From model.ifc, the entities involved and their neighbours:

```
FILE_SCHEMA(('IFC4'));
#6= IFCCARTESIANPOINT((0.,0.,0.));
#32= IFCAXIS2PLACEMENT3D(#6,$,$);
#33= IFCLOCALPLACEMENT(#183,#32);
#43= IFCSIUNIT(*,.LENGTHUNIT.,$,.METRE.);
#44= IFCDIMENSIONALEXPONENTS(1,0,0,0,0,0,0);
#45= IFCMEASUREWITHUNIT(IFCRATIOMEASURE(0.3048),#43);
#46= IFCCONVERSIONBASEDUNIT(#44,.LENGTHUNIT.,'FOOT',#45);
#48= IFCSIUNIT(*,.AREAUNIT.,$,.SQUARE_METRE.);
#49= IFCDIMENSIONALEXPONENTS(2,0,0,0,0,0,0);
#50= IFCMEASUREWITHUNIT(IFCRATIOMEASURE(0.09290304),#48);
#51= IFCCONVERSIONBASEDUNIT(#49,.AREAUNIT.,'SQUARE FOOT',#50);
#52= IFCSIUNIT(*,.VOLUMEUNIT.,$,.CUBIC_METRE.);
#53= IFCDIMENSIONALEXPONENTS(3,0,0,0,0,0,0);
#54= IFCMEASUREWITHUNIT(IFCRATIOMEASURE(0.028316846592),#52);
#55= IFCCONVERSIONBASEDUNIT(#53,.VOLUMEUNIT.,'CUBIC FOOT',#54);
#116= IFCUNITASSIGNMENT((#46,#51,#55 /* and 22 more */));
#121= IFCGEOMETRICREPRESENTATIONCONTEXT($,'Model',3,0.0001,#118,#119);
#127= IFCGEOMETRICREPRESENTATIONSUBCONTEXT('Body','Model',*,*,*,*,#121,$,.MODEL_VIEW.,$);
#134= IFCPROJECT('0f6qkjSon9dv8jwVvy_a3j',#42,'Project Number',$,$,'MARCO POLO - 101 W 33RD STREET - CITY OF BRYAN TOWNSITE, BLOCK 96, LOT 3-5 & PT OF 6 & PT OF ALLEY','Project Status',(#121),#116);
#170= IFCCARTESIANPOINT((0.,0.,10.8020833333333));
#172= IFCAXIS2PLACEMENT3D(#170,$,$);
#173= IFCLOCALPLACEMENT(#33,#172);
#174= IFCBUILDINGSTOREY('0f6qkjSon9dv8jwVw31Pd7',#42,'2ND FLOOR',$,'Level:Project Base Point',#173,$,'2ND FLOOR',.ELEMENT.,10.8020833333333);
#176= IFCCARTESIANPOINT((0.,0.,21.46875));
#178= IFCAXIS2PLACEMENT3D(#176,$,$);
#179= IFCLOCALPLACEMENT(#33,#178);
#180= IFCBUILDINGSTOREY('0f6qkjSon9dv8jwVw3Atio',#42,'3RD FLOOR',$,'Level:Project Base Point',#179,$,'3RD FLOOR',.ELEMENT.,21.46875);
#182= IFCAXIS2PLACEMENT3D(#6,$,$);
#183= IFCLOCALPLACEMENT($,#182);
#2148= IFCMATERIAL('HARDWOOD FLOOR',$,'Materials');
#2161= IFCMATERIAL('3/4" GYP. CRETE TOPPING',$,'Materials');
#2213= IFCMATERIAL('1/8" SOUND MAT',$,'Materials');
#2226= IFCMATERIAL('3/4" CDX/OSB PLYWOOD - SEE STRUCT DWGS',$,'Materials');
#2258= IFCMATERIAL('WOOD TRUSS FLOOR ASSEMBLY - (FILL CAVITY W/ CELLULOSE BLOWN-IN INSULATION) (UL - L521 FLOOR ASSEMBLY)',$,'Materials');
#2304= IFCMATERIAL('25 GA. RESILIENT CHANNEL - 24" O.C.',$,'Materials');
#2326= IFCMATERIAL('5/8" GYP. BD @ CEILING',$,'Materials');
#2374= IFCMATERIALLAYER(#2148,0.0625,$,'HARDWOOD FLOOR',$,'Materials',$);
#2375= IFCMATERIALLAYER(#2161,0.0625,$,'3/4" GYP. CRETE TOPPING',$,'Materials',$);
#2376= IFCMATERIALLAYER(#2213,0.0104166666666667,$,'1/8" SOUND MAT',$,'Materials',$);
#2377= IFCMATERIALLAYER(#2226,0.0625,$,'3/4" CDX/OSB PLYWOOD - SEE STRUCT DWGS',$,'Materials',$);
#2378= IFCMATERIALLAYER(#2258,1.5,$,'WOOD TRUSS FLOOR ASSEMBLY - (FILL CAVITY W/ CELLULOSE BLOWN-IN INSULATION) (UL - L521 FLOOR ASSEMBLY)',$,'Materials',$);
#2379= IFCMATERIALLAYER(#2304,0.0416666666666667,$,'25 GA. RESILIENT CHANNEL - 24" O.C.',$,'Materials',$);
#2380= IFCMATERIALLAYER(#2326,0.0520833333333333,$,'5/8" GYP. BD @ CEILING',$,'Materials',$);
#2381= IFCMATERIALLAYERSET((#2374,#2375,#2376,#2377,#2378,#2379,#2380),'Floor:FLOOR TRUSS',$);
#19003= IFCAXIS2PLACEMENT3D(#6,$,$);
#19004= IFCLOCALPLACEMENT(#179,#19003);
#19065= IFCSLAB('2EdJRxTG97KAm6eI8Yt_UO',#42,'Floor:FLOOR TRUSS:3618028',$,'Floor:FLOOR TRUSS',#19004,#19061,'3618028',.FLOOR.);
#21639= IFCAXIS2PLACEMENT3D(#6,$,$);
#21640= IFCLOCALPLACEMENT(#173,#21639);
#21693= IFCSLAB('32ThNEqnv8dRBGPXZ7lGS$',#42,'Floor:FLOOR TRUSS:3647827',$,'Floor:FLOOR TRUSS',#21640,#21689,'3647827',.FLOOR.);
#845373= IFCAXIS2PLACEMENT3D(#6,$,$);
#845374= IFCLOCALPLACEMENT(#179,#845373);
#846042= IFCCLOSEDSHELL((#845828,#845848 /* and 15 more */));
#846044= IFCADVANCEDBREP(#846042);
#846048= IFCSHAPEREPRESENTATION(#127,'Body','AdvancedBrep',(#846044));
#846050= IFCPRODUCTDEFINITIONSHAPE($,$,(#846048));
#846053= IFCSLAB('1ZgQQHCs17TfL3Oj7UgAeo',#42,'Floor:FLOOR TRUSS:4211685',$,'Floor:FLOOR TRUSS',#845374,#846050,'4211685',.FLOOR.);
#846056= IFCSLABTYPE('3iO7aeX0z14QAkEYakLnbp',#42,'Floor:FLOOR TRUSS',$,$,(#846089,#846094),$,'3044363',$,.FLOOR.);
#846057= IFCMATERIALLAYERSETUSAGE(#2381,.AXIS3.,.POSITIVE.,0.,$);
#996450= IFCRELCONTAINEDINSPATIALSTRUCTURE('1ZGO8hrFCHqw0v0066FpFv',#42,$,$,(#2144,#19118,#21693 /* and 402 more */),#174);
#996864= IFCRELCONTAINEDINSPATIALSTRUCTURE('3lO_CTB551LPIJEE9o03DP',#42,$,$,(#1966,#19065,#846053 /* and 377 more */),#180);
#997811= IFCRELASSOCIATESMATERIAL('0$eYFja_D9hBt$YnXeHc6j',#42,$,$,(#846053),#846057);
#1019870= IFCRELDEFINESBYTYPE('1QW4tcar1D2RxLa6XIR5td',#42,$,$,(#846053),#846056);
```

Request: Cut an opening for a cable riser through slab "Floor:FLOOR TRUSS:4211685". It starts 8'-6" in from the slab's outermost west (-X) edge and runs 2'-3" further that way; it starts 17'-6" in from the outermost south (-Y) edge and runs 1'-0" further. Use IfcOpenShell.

```python
import numpy as np
import ifcopenshell
import ifcopenshell.api.feature
import ifcopenshell.api.geometry
import ifcopenshell.api.root
import ifcopenshell.geom
import ifcopenshell.util.placement
import ifcopenshell.util.representation
import ifcopenshell.util.shape
import ifcopenshell.util.unit

model = ifcopenshell.open("model.ifc")
unit_scale = ifcopenshell.util.unit.calculate_unit_scale(model)
settings = ifcopenshell.geom.settings()


def volume(element):
    """Net volume in cubic metres, openings subtracted."""
    shape = ifcopenshell.geom.create_shape(settings, element)
    return ifcopenshell.util.shape.get_volume(shape.geometry)


slab = model.by_guid("1ZgQQHCs17TfL3Oj7UgAeo")
before = volume(slab)

# Extent in the slab's own axes, in metres. The edges named are its -X and -Y sides.
slab_shape = ifcopenshell.geom.create_shape(settings, slab)
vertices = ifcopenshell.util.shape.get_vertices(slab_shape.geometry)
x_min, y_min, bottom = vertices.min(axis=0)
top = vertices[:, 2].max()

opening = ifcopenshell.api.root.create_entity(model, ifc_class="IfcOpeningElement", name="Cable riser opening", predefined_type="OPENING")
context = ifcopenshell.util.representation.get_context(model, "Model", "Body", "MODEL_VIEW")
width, depth = 0.6858, 0.3048
outline = [(0.0, 0.0), (width, 0.0), (width, depth), (0.0, depth), (0.0, 0.0)]
# Overshoot both faces by 50 mm so the cut is clean.
shape = ifcopenshell.api.geometry.add_slab_representation(
    model, context=context, depth=top - bottom + 0.1, polyline=outline
)
ifcopenshell.api.geometry.assign_representation(model, product=opening, representation=shape)

matrix = ifcopenshell.util.placement.get_local_placement(slab.ObjectPlacement)
matrix[:, 3] = matrix @ np.append(np.array([x_min + 2.5908, y_min + 5.334, bottom - 0.05]) / unit_scale, 1.0)
ifcopenshell.api.geometry.edit_object_placement(model, product=opening, matrix=matrix, is_si=False)
ifcopenshell.api.feature.add_feature(model, feature=opening, element=slab)

after = volume(slab)

print(f"slab volume {before:.3f} -> {after:.3f} m3")

model.write("model_edited.ifc")
```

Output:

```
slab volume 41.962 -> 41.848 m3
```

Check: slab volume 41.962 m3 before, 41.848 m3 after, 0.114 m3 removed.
